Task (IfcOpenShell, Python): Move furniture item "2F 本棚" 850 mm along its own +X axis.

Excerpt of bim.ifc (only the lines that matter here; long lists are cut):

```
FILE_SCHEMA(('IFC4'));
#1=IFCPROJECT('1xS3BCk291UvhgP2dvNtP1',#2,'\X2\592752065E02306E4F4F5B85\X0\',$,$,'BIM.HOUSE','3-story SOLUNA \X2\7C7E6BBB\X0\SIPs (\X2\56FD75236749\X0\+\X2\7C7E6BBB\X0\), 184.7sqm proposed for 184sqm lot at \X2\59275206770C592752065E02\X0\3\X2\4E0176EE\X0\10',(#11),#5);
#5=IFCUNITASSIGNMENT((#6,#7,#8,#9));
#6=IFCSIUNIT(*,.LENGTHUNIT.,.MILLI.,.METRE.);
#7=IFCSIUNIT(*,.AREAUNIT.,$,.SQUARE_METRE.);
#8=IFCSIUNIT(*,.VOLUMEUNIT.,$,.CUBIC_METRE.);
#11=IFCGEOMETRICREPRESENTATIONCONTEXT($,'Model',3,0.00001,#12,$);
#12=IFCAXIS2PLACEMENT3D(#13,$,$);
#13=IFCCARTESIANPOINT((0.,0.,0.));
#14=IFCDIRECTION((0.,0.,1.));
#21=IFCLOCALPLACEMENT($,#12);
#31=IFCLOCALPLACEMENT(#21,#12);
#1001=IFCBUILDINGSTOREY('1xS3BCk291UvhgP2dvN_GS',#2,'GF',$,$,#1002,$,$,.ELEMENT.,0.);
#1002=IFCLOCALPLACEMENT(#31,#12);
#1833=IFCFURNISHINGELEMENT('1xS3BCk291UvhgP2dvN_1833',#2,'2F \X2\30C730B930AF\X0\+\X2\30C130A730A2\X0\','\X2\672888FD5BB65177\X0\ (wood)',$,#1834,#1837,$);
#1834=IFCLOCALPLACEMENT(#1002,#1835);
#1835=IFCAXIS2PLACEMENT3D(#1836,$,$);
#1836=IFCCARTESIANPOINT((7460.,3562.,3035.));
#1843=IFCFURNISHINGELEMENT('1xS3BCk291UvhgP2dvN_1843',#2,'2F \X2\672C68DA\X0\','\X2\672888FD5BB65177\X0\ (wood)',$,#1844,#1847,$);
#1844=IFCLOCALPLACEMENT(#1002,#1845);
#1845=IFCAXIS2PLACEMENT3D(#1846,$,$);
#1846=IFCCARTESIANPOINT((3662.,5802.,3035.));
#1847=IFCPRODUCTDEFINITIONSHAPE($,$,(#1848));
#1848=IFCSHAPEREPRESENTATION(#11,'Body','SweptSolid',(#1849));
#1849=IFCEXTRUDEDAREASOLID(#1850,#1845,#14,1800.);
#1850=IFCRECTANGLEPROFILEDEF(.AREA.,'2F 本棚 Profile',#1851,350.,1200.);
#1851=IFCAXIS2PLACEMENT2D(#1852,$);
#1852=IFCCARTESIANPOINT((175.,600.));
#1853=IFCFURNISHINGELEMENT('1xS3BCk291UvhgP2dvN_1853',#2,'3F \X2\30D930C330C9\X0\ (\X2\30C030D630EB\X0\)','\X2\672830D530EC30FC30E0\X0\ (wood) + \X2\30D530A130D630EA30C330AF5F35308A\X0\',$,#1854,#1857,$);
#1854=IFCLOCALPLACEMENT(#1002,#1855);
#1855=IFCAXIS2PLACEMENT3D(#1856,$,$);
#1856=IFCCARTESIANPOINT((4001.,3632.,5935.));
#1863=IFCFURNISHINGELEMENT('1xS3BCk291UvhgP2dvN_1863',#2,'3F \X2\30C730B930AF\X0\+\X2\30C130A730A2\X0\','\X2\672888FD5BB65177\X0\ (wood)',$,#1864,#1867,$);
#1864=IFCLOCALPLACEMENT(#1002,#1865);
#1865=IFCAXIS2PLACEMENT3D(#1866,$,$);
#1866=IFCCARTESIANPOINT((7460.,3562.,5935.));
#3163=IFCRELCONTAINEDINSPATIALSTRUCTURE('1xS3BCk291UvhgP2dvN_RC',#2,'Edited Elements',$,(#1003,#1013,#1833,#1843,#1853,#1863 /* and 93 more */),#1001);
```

```python
import ifcopenshell
import ifcopenshell.api.geometry
import ifcopenshell.util.placement

model = ifcopenshell.open("bim.ifc")

item = model.by_guid("1xS3BCk291UvhgP2dvN_1843")
matrix = ifcopenshell.util.placement.get_local_placement(item.ObjectPlacement)
matrix[:3, 3] += matrix[:3, 0] * 850.0
ifcopenshell.api.geometry.edit_object_placement(model, product=item, matrix=matrix, is_si=False)

print(ifcopenshell.util.placement.get_local_placement(item.ObjectPlacement).round(3) + 0.0)

model.write("bim_edited.ifc")
```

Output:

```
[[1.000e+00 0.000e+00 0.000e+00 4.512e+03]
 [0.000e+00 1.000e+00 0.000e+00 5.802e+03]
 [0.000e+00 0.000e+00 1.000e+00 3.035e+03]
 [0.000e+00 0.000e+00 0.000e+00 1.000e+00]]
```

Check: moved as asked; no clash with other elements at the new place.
